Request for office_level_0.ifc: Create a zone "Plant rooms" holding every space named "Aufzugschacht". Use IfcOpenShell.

First a look at what the model holds.

```python
import ifcopenshell

model = ifcopenshell.open("office_level_0.ifc")
print(model.schema)
seen = {}
for space in model.by_type("IfcSpace"):
    seen[space.LongName] = seen.get(space.LongName, 0) + 1
for name, count in sorted(seen.items(), key=str):
    print(count, "x", name)
print("zones:", [z.Name for z in model.by_type("IfcZone")][:20])
```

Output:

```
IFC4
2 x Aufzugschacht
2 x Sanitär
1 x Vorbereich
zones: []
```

```python
import ifcopenshell
import ifcopenshell.api.group
import ifcopenshell.api.root

model = ifcopenshell.open("office_level_0.ifc")

names = {"Aufzugschacht"}
spaces = [s for s in model.by_type("IfcSpace") if s.LongName in names]

zone = ifcopenshell.api.root.create_entity(model, ifc_class="IfcZone", name="Plant rooms")
ifcopenshell.api.group.assign_group(model, products=spaces, group=zone)
print(len(spaces), "spaces in", zone.Name)

model.write("office_level_0_edited.ifc")
```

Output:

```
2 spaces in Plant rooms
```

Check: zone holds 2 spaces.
